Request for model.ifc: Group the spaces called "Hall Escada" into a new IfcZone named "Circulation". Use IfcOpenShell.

First a look at what the model holds.

```python
import ifcopenshell

model = ifcopenshell.open("model.ifc")
print(model.schema)
seen = {}
for space in model.by_type("IfcSpace"):
    seen[space.LongName] = seen.get(space.LongName, 0) + 1
for name, count in sorted(seen.items(), key=str):
    print(count, "x", name)
print("zones:", [z.Name for z in model.by_type("IfcZone")][:20])
```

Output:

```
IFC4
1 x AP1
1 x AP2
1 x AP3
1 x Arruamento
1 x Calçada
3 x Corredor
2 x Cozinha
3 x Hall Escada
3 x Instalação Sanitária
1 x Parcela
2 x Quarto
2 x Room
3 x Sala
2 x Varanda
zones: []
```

```python
import ifcopenshell
import ifcopenshell.api.group
import ifcopenshell.api.root

model = ifcopenshell.open("model.ifc")

names = {"Hall Escada"}
spaces = [s for s in model.by_type("IfcSpace") if s.LongName in names]

zone = ifcopenshell.api.root.create_entity(model, ifc_class="IfcZone", name="Circulation")
ifcopenshell.api.group.assign_group(model, products=spaces, group=zone)
print(len(spaces), "spaces in", zone.Name)

model.write("model_rev.ifc")
```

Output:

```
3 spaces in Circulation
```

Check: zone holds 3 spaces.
